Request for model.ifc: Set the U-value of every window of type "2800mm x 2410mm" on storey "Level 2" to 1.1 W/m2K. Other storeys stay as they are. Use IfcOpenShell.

First a look at what the model holds.

```python
import ifcopenshell
import ifcopenshell.util.element

model = ifcopenshell.open("model.ifc")
print(model.schema)
storey = next(s for s in model.by_type("IfcBuildingStorey") if s.Name == "Level 2")
windows = [e for e in ifcopenshell.util.element.get_decomposition(storey) if e.is_a("IfcWindow")]
seen = {}
for e in windows:
    element_type = ifcopenshell.util.element.get_type(e)
    key = (element_type.Name if element_type != e and element_type else None, ifcopenshell.util.element.get_pset(e, "Pset_WindowCommon", "ThermalTransmittance"))
    seen[key] = seen.get(key, 0) + 1
for (name, value), count in sorted(seen.items(), key=str):
    print(count, "x", name, "|", value)
```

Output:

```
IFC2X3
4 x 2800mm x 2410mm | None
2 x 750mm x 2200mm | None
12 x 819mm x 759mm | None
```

```python
import ifcopenshell
import ifcopenshell.api.pset
import ifcopenshell.util.element

model = ifcopenshell.open("model.ifc")

storey = next(s for s in model.by_type("IfcBuildingStorey") if s.Name == "Level 2")
windows = [e for e in ifcopenshell.util.element.get_decomposition(storey) if e.is_a("IfcWindow")]

count = 0
for e in windows:
    element_type = ifcopenshell.util.element.get_type(e)
    if element_type in (None, e) or element_type.Name != "2800mm x 2410mm":
        continue
    # add_pset returns the element's existing set when there is one.
    pset = ifcopenshell.api.pset.add_pset(model, product=e, name="Pset_WindowCommon")
    ifcopenshell.api.pset.edit_pset(model, pset=pset, properties={"ThermalTransmittance": 1.1})
    count += 1

print(count, "windows updated")

model.write("model_edited.ifc")
```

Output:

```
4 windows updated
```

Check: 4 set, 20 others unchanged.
